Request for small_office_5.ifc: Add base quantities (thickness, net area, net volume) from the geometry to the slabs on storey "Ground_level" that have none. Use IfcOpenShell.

First a look at what the model holds.

```python
import ifcopenshell
import ifcopenshell.util.element
import ifcopenshell.util.unit

model = ifcopenshell.open("small_office_5.ifc")
print(model.schema)
for unit_type in ("LENGTHUNIT", "AREAUNIT", "VOLUMEUNIT"):
    print(unit_type, ifcopenshell.util.unit.calculate_unit_scale(model, unit_type))
storey = next(s for s in model.by_type("IfcBuildingStorey") if s.Name == "Ground_level")
slabs = [e for e in ifcopenshell.util.element.get_decomposition(storey) if e.is_a("IfcSlab")]
for e in sorted(slabs, key=lambda e: e.id()):
    print(e.id(), e.is_a(), e.Name, list(ifcopenshell.util.element.get_psets(e, qtos_only=True)), sep=" | ")
```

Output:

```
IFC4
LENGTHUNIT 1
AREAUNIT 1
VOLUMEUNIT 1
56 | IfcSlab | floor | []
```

```python
import ifcopenshell
import ifcopenshell.api.pset
import ifcopenshell.geom
import ifcopenshell.util.element
import ifcopenshell.util.shape
import ifcopenshell.util.unit

model = ifcopenshell.open("small_office_5.ifc")
unit_scale = ifcopenshell.util.unit.calculate_unit_scale(model)
area_scale = ifcopenshell.util.unit.calculate_unit_scale(model, "AREAUNIT")
volume_scale = ifcopenshell.util.unit.calculate_unit_scale(model, "VOLUMEUNIT")
settings = ifcopenshell.geom.settings()

storey = next(s for s in model.by_type("IfcBuildingStorey") if s.Name == "Ground_level")
slabs = [e for e in ifcopenshell.util.element.get_decomposition(storey) if e.is_a("IfcSlab")]

for e in sorted(slabs, key=lambda e: e.id()):
    if ifcopenshell.util.element.get_psets(e, qtos_only=True, should_inherit=False):
        continue
    # Geometry comes back in metres, in the element's own axes.
    shape = ifcopenshell.geom.create_shape(settings, e)
    values = {
        "Width": ifcopenshell.util.shape.get_z(shape.geometry) / unit_scale,
        "NetArea": ifcopenshell.util.shape.get_footprint_area(shape.geometry) / area_scale,
        "NetVolume": ifcopenshell.util.shape.get_volume(shape.geometry) / volume_scale,
    }
    qto = ifcopenshell.api.pset.add_qto(model, product=e, name="Qto_SlabBaseQuantities")
    ifcopenshell.api.pset.edit_qto(model, qto=qto, properties=values)
    print(e.id(), {k: round(v, 3) for k, v in values.items()})

model.write("small_office_5_rev.ifc")
```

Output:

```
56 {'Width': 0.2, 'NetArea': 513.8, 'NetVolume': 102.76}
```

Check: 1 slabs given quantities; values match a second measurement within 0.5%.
